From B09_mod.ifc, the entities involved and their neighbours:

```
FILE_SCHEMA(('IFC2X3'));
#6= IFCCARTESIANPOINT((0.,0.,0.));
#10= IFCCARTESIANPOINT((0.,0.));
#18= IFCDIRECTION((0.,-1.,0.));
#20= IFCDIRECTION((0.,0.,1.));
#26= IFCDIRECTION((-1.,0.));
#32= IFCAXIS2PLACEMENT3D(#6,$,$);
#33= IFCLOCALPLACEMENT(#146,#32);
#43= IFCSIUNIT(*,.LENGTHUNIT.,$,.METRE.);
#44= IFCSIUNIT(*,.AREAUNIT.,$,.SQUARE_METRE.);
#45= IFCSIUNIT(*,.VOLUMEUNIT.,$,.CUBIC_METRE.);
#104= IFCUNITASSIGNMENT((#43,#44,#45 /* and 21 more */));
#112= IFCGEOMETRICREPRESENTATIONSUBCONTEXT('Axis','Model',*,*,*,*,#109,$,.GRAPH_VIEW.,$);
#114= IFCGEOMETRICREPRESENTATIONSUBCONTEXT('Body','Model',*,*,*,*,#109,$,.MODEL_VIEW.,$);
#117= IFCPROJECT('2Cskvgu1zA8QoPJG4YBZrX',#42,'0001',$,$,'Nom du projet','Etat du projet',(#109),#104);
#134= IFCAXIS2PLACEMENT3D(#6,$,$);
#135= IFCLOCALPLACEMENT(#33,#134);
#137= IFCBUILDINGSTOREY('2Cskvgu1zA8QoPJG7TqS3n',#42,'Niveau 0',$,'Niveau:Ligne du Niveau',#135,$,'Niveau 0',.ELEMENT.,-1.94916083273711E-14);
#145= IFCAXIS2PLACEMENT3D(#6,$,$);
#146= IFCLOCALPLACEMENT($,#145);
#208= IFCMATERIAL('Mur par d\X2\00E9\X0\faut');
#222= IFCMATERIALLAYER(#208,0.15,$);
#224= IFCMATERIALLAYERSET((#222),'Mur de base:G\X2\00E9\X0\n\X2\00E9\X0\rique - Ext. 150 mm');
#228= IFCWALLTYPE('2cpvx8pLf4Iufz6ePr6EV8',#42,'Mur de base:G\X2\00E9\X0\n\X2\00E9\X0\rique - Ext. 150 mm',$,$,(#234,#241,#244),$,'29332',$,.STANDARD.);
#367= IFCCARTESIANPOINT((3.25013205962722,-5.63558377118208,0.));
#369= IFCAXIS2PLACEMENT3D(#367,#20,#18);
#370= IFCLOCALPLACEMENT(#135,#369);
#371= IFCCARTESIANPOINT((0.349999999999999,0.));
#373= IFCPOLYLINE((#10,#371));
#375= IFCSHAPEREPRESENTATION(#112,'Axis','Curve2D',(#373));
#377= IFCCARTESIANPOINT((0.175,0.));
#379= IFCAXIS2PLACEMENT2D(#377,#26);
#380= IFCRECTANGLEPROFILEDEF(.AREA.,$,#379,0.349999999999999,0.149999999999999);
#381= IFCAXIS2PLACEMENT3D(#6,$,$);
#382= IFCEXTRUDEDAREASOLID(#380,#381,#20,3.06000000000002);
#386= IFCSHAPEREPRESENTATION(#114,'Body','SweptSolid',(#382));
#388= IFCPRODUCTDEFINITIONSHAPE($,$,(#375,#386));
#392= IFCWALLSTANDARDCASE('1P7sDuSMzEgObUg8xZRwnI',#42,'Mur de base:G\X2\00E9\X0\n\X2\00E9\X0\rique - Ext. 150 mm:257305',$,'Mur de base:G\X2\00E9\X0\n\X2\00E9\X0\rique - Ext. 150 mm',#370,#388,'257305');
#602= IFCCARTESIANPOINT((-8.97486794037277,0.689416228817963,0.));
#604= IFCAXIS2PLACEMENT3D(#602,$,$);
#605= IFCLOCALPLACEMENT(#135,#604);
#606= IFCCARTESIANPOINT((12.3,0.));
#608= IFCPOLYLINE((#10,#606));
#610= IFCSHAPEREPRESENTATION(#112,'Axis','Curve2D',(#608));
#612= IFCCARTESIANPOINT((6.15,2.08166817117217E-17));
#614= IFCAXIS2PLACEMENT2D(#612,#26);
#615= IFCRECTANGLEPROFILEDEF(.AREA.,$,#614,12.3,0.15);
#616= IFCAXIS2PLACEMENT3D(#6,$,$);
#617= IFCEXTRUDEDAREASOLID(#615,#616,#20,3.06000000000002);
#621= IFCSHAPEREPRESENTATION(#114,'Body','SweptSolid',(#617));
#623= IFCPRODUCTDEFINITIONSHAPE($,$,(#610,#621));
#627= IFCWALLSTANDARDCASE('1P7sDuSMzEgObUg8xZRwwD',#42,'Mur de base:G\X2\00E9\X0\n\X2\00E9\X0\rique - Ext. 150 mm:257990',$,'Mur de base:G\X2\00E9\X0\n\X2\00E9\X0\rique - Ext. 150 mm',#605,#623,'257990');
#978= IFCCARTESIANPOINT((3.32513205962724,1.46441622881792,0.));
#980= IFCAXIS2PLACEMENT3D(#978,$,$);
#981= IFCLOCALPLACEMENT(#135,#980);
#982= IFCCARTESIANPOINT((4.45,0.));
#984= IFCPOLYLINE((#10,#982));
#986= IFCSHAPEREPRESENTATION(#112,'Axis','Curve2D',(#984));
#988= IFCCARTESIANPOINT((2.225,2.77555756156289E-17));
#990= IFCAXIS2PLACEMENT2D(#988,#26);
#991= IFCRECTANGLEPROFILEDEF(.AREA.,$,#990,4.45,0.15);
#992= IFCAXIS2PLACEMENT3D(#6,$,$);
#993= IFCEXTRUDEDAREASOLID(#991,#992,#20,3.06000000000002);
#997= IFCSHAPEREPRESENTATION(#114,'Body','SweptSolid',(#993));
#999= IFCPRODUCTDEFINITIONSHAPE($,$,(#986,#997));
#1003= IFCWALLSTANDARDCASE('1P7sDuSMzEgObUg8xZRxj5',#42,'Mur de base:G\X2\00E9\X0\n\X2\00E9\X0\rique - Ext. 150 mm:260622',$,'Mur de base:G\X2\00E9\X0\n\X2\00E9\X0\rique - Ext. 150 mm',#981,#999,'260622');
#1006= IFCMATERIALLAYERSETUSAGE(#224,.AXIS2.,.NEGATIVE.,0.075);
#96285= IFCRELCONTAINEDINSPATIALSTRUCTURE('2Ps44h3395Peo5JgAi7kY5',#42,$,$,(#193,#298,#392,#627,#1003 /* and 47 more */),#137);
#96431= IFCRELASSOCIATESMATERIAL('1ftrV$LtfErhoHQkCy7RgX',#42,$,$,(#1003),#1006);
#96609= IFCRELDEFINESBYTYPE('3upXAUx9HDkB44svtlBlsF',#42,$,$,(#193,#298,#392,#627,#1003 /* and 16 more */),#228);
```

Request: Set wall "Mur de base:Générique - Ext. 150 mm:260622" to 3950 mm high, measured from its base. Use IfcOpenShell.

```python
import ifcopenshell
import ifcopenshell.geom
import ifcopenshell.util.representation
import ifcopenshell.util.shape
import ifcopenshell.util.unit

model = ifcopenshell.open("B09_mod.ifc")
unit_scale = ifcopenshell.util.unit.calculate_unit_scale(model)
settings = ifcopenshell.geom.settings()


def volume(element):
    """Net volume in cubic metres, openings subtracted."""
    shape = ifcopenshell.geom.create_shape(settings, element)
    return ifcopenshell.util.shape.get_volume(shape.geometry)


wall = model.by_guid("1P7sDuSMzEgObUg8xZRxj5")
before = volume(wall)

body = ifcopenshell.util.representation.get_representation(wall, "Model", "Body")
solid = body.Items[0]
old_height = solid.Depth
solid.Depth = 3.95 / unit_scale
after = volume(wall)

print(f"height {old_height:g} -> {solid.Depth:g}, volume {before:.3f} -> {after:.3f} m3")

model.write("B09_mod_updated.ifc")
```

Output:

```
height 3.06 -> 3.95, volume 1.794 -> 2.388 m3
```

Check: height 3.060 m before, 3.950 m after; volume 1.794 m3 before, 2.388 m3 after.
